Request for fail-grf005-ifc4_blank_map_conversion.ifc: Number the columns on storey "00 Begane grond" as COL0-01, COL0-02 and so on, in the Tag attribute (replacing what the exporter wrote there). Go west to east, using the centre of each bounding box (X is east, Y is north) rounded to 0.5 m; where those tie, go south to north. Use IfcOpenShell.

First a look at what the model holds.

```python
import ifcopenshell
import ifcopenshell.util.element
import ifcopenshell.util.placement

model = ifcopenshell.open("fail-grf005-ifc4_blank_map_conversion.ifc")
print(model.schema)
storey = next(s for s in model.by_type("IfcBuildingStorey") if s.Name == "00 Begane grond")
columns = [e for e in ifcopenshell.util.element.get_decomposition(storey) if e.is_a("IfcColumn")]
for e in sorted(columns, key=lambda e: e.id()):
    origin = ifcopenshell.util.placement.get_local_placement(e.ObjectPlacement)[:3, 3]
    print(e.id(), e.Tag, e.Name, origin.round(2) + 0.0, sep=" | ")
```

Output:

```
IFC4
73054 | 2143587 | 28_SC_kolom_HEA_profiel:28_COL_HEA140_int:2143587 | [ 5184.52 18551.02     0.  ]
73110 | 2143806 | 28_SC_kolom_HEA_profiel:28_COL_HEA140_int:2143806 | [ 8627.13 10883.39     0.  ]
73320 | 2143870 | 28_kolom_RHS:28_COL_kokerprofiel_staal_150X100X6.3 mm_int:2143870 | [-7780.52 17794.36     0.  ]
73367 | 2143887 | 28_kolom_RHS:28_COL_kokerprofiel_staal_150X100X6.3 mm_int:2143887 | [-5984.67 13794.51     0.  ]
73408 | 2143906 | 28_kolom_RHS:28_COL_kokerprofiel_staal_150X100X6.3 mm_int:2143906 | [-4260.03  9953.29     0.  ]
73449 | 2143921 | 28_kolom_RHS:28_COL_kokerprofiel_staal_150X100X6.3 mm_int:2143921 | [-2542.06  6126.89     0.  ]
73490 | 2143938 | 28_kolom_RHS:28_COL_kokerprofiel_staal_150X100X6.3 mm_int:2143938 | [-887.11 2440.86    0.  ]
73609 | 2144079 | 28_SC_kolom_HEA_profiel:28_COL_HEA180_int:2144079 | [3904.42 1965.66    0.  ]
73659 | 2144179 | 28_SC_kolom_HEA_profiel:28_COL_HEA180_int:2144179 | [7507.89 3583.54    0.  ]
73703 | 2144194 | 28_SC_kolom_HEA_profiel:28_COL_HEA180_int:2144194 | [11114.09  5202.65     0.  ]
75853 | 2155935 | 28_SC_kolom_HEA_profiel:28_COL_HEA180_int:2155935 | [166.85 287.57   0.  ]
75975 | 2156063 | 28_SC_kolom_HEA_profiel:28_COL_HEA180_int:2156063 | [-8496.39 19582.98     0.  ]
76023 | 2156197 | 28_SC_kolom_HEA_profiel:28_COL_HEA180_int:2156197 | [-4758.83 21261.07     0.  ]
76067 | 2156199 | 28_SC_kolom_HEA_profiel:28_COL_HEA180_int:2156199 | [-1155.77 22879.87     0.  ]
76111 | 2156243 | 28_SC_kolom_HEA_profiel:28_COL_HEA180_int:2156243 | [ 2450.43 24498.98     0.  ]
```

```python
import ifcopenshell
import ifcopenshell.geom
import ifcopenshell.util.element
import ifcopenshell.util.shape

model = ifcopenshell.open("fail-grf005-ifc4_blank_map_conversion.ifc")
settings = ifcopenshell.geom.settings()
settings.set("use-world-coords", True)


def centre(element):
    shape = ifcopenshell.geom.create_shape(settings, element)
    return ifcopenshell.util.shape.get_bbox_centroid(shape.geometry)


storey = next(s for s in model.by_type("IfcBuildingStorey") if s.Name == "00 Begane grond")
columns = [e for e in ifcopenshell.util.element.get_decomposition(storey) if e.is_a("IfcColumn")]

# Insertion points can sit at a corner or the storey origin, so sort by the geometry (in metres).
centres = {e: centre(e) for e in columns}
columns.sort(key=lambda e: (round(centres[e][0] / 0.5), centres[e][1]))

for i, e in enumerate(columns, start=1):
    number = f"COL0-{i:02d}"
    e.Tag = number
    print(e.id(), number)

model.write("fail-grf005-ifc4_blank_map_conversion-out.ifc")
```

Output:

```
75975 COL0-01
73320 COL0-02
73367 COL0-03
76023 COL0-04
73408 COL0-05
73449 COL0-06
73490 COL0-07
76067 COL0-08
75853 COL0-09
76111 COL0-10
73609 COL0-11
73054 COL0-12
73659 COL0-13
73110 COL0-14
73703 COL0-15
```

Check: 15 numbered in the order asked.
